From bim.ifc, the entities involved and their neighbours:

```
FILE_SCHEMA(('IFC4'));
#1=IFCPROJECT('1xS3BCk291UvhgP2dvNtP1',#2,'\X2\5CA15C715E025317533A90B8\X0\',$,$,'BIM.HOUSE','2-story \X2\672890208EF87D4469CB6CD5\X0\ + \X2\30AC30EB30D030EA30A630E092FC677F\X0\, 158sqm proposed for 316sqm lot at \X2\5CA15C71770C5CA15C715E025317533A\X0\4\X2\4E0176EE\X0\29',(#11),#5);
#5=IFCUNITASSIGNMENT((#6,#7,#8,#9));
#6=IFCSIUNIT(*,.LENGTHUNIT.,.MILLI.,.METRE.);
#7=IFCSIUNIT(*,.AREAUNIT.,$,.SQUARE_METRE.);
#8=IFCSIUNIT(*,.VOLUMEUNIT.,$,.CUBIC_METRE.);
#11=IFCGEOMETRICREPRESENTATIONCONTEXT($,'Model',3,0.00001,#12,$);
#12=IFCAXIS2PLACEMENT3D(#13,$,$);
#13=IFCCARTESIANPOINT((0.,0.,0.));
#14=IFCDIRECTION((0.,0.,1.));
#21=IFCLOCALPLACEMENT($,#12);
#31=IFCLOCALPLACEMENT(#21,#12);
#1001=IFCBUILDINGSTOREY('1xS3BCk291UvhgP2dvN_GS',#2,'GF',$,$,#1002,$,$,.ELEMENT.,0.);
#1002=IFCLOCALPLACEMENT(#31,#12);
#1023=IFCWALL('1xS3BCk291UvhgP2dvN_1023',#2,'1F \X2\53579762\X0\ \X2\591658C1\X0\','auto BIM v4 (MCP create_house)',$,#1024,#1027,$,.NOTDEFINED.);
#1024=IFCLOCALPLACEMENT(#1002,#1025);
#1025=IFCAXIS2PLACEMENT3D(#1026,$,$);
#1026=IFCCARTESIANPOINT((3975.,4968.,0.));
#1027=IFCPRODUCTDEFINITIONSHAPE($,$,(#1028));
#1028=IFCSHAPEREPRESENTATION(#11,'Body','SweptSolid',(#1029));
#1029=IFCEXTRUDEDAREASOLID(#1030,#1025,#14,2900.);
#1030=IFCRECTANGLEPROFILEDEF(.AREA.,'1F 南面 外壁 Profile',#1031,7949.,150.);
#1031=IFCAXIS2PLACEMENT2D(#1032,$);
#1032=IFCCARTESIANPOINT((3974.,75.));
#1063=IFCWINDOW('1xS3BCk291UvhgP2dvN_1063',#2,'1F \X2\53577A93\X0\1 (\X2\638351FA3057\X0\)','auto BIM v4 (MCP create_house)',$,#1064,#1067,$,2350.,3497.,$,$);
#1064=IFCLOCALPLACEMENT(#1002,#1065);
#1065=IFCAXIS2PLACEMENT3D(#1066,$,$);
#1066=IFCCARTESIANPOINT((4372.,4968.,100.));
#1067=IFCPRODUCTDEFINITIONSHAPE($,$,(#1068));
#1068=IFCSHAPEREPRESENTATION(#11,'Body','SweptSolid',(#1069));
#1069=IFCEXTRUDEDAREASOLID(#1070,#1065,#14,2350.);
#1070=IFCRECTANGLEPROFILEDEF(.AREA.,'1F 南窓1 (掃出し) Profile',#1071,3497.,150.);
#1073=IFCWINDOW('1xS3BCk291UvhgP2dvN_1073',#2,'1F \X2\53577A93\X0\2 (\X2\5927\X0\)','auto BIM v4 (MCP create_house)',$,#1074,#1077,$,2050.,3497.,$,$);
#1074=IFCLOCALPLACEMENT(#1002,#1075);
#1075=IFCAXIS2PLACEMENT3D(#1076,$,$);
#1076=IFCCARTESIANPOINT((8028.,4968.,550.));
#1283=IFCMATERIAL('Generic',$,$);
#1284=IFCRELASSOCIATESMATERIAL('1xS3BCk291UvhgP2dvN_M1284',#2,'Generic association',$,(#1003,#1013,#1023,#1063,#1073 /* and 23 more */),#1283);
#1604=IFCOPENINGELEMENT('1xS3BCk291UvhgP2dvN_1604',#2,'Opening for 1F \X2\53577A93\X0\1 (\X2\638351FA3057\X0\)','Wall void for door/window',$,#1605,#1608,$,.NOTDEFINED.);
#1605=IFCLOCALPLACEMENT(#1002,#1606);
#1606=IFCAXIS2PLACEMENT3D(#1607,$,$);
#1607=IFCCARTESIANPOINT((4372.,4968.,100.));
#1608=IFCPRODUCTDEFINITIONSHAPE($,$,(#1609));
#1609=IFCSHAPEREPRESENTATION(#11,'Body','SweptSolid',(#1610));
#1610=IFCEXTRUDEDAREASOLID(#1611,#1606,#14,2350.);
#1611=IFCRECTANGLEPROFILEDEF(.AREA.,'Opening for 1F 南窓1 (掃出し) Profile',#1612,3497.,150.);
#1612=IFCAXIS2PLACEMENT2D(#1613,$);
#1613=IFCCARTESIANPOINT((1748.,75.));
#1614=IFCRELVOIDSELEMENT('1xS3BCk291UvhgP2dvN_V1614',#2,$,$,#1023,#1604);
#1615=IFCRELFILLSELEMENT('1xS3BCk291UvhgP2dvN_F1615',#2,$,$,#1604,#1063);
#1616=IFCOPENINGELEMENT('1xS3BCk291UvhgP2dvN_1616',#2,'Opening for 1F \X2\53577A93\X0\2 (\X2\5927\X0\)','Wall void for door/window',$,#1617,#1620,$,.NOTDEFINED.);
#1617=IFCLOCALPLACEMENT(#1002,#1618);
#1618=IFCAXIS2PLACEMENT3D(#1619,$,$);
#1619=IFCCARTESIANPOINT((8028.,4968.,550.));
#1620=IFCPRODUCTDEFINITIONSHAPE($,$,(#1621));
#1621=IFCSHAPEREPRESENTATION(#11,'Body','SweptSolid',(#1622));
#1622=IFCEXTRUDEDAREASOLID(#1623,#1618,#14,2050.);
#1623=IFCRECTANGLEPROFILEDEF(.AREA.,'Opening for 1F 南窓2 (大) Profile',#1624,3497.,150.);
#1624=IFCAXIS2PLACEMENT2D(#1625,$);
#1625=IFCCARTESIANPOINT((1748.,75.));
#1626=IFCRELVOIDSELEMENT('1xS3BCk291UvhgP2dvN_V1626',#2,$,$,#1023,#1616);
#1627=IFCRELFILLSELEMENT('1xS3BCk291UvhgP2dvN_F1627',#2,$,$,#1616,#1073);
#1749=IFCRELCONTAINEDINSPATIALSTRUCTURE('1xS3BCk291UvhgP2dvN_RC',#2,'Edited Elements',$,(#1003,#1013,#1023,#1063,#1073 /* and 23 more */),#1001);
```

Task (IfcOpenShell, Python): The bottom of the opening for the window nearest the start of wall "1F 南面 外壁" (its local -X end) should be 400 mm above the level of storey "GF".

```python
import numpy as np
import ifcopenshell
import ifcopenshell.api.geometry
import ifcopenshell.geom
import ifcopenshell.util.element
import ifcopenshell.util.placement
import ifcopenshell.util.shape
import ifcopenshell.util.unit

model = ifcopenshell.open("bim.ifc")
unit_scale = ifcopenshell.util.unit.calculate_unit_scale(model)

window = model.by_id(1063)
opening = window.FillsVoids[0].RelatingOpeningElement
storey = ifcopenshell.util.element.get_container(window, ifc_class="IfcBuildingStorey")
level = ifcopenshell.util.placement.get_local_placement(storey.ObjectPlacement)[2, 3]

# The opening's origin need not be at the sill, so measure its lowest point.
shape = ifcopenshell.geom.create_shape(ifcopenshell.geom.settings(), opening)
bottom = ifcopenshell.util.shape.get_shape_bottom_elevation(shape, shape.geometry) / unit_scale
dz = level + 400.0 - bottom

shift = np.array([0.0, 0.0, dz])
# The window is not placed relative to its opening, so move both.
for product in (opening, window):
    matrix = ifcopenshell.util.placement.get_local_placement(product.ObjectPlacement)
    matrix[:3, 3] += shift
    ifcopenshell.api.geometry.edit_object_placement(model, product=product, matrix=matrix, is_si=False)

print(f"moved by {dz * unit_scale:+.3f} m")

model.write("bim-out.ifc")
```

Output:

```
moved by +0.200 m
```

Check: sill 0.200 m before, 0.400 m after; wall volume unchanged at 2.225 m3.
